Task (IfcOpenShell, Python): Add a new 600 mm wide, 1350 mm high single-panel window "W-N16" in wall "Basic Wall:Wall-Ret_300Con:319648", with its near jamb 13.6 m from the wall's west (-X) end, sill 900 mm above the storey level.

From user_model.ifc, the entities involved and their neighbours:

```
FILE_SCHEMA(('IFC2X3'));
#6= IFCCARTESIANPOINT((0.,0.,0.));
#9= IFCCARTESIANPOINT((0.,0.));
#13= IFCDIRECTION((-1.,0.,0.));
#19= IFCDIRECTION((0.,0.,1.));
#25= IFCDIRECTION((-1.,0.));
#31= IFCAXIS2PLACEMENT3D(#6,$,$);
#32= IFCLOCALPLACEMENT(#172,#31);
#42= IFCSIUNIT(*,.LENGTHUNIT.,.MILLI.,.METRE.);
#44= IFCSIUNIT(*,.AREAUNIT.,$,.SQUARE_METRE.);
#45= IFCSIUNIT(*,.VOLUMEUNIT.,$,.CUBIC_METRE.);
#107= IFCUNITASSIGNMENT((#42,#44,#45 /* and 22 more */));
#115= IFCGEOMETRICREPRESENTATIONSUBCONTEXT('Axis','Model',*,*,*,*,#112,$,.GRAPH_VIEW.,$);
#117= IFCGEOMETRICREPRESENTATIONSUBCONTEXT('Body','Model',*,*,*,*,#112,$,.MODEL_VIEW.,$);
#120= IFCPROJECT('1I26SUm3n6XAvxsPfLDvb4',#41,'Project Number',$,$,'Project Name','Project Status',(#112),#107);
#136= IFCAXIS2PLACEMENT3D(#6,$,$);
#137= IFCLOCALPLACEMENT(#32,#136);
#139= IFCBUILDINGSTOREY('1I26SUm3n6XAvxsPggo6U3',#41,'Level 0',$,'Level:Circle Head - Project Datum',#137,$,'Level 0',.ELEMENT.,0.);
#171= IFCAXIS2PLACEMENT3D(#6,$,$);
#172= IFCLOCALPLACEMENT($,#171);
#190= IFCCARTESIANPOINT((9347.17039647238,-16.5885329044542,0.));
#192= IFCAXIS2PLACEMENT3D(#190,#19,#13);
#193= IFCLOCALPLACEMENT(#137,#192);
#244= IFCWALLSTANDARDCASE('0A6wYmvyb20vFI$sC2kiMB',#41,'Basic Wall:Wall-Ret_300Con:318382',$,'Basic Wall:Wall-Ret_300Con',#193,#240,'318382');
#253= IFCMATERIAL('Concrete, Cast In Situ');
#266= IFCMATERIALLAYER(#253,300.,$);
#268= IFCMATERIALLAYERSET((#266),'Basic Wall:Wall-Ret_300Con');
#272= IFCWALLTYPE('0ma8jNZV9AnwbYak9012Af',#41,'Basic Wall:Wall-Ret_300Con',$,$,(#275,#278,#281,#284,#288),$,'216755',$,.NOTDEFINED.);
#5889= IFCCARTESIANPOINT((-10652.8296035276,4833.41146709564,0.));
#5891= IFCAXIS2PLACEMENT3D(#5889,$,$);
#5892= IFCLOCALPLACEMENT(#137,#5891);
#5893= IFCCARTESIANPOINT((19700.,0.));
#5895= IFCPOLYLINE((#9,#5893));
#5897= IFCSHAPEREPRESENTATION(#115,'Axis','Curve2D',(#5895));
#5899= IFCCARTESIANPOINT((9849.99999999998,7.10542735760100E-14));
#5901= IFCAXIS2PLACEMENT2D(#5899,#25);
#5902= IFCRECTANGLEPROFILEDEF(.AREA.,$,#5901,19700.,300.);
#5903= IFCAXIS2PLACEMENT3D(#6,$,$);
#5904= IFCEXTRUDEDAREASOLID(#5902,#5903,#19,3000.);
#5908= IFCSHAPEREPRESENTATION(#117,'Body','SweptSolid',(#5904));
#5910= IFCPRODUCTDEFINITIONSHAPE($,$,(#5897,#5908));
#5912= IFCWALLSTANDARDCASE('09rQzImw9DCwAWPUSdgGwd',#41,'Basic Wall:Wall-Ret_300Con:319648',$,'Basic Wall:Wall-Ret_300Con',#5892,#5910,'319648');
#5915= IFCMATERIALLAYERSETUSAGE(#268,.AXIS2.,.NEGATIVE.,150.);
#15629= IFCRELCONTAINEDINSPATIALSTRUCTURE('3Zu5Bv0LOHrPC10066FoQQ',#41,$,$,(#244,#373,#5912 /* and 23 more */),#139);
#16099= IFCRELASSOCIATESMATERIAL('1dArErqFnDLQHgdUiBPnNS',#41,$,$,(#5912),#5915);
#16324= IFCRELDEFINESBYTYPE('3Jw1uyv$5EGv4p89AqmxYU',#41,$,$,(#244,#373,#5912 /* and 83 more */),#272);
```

```python
import numpy as np
import ifcopenshell
import ifcopenshell.api.feature
import ifcopenshell.api.geometry
import ifcopenshell.api.root
import ifcopenshell.api.spatial
import ifcopenshell.api.type
import ifcopenshell.geom
import ifcopenshell.util.element
import ifcopenshell.util.placement
import ifcopenshell.util.representation
import ifcopenshell.util.shape
import ifcopenshell.util.unit

model = ifcopenshell.open("user_model.ifc")
unit_scale = ifcopenshell.util.unit.calculate_unit_scale(model)
settings = ifcopenshell.geom.settings()


def volume(element):
    """Net volume in cubic metres, openings subtracted."""
    shape = ifcopenshell.geom.create_shape(settings, element)
    return ifcopenshell.util.shape.get_volume(shape.geometry)


wall = model.by_id(5912)
storey = ifcopenshell.util.element.get_container(wall, ifc_class="IfcBuildingStorey")
context = ifcopenshell.util.representation.get_context(model, "Model", "Body", "MODEL_VIEW")
before = volume(wall)

width, height, from_end, sill = 0.6, 1.35, 13.6, 0.9  # metres

# The wall runs along its own X axis, and the end named is its -X end.
wall_shape = ifcopenshell.geom.create_shape(settings, wall)
x, y, z = ifcopenshell.util.shape.get_vertices(wall_shape.geometry).T
start = x.min() + from_end
face, thickness = float(y.min()), float(y.max() - y.min())
wall_matrix = ifcopenshell.util.placement.get_local_placement(wall.ObjectPlacement)
level = ifcopenshell.util.placement.get_local_placement(storey.ObjectPlacement)[2, 3]


def in_wall(x, y):
    """Placement at x, y metres in the wall's axes, at sill height."""
    matrix = wall_matrix.copy()
    matrix[:, 3] = wall_matrix @ np.array([x / unit_scale, y / unit_scale, 0.0, 1.0])
    matrix[2, 3] = level + sill / unit_scale
    return matrix


# Opening: a box that overshoots both wall faces by 50 mm.
opening = ifcopenshell.api.root.create_entity(model, ifc_class="IfcOpeningElement")
box = ifcopenshell.api.geometry.add_wall_representation(
    model, context=context, length=width, height=height, thickness=thickness + 0.1
)
ifcopenshell.api.geometry.assign_representation(model, product=opening, representation=box)
ifcopenshell.api.geometry.edit_object_placement(model, product=opening, matrix=in_wall(start, face - 0.05), is_si=False)
ifcopenshell.api.feature.add_feature(model, feature=opening, element=wall)

window = ifcopenshell.api.root.create_entity(model, ifc_class="IfcWindow", name="W-N16")
window.OverallWidth, window.OverallHeight = width / unit_scale, height / unit_scale
body = ifcopenshell.api.geometry.add_window_representation(
    model,
    context=context,
    overall_width=window.OverallWidth,
    overall_height=window.OverallHeight,
    partition_type="SINGLE_PANEL",
)
ifcopenshell.api.geometry.assign_representation(model, product=window, representation=body)
ifcopenshell.api.spatial.assign_container(model, products=[window], relating_structure=storey)
fills = ifcopenshell.api.feature.add_filling(model, opening=opening, element=window)
fills.OwnerHistory = window.OwnerHistory  # required in IFC2X3

# IFC2X3 keeps the operation on the window style.
style = ifcopenshell.api.root.create_entity(model, ifc_class="IfcWindowStyle", name="W-N16")
style.OperationType, style.ConstructionType = "SINGLE_PANEL", "NOTDEFINED"
style.ParameterTakesPrecedence = style.Sizeable = False
ifcopenshell.api.type.assign_type(model, related_objects=[window], relating_type=style)

# Centre the window in the wall's thickness.
ifcopenshell.api.geometry.edit_object_placement(model, product=window, matrix=in_wall(start, face), is_si=False)
window_shape = ifcopenshell.geom.create_shape(settings, window)
depth = ifcopenshell.util.shape.get_vertices(window_shape.geometry)[:, 1]
offset = face + thickness / 2 - (depth.min() + depth.max()) / 2
ifcopenshell.api.geometry.edit_object_placement(model, product=window, matrix=in_wall(start, offset), is_si=False)

after = volume(wall)

print(f"wall volume {before:.3f} -> {after:.3f} m3")

model.write("user_model_rev.ifc")
```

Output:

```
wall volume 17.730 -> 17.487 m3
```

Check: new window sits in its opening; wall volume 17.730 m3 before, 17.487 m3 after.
